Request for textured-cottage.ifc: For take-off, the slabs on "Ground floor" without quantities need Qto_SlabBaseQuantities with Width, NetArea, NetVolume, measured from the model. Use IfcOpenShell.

First a look at what the model holds.

```python
import ifcopenshell
import ifcopenshell.util.element
import ifcopenshell.util.unit

model = ifcopenshell.open("textured-cottage.ifc")
print(model.schema)
for unit_type in ("LENGTHUNIT", "AREAUNIT", "VOLUMEUNIT"):
    print(unit_type, ifcopenshell.util.unit.calculate_unit_scale(model, unit_type))
storey = next(s for s in model.by_type("IfcBuildingStorey") if s.Name == "Ground floor")
slabs = [e for e in ifcopenshell.util.element.get_decomposition(storey) if e.is_a("IfcSlab")]
for e in sorted(slabs, key=lambda e: e.id()):
    print(e.id(), e.is_a(), e.Name, list(ifcopenshell.util.element.get_psets(e, qtos_only=True)), sep=" | ")
```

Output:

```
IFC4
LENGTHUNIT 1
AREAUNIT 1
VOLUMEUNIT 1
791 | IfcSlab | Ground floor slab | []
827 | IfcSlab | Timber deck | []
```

```python
import ifcopenshell
import ifcopenshell.api.pset
import ifcopenshell.geom
import ifcopenshell.util.element
import ifcopenshell.util.shape
import ifcopenshell.util.unit

model = ifcopenshell.open("textured-cottage.ifc")
unit_scale = ifcopenshell.util.unit.calculate_unit_scale(model)
area_scale = ifcopenshell.util.unit.calculate_unit_scale(model, "AREAUNIT")
volume_scale = ifcopenshell.util.unit.calculate_unit_scale(model, "VOLUMEUNIT")
settings = ifcopenshell.geom.settings()

storey = next(s for s in model.by_type("IfcBuildingStorey") if s.Name == "Ground floor")
slabs = [e for e in ifcopenshell.util.element.get_decomposition(storey) if e.is_a("IfcSlab")]

for e in sorted(slabs, key=lambda e: e.id()):
    if ifcopenshell.util.element.get_psets(e, qtos_only=True, should_inherit=False):
        continue
    # Geometry comes back in metres, in the element's own axes.
    shape = ifcopenshell.geom.create_shape(settings, e)
    values = {
        "Width": ifcopenshell.util.shape.get_z(shape.geometry) / unit_scale,
        "NetArea": ifcopenshell.util.shape.get_footprint_area(shape.geometry) / area_scale,
        "NetVolume": ifcopenshell.util.shape.get_volume(shape.geometry) / volume_scale,
    }
    qto = ifcopenshell.api.pset.add_qto(model, product=e, name="Qto_SlabBaseQuantities")
    ifcopenshell.api.pset.edit_qto(model, qto=qto, properties=values)
    print(e.id(), {k: round(v, 3) for k, v in values.items()})

model.write("textured-cottage_updated.ifc")
```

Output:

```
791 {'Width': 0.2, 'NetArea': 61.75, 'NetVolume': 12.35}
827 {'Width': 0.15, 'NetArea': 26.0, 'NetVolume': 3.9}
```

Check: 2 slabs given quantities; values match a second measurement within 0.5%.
